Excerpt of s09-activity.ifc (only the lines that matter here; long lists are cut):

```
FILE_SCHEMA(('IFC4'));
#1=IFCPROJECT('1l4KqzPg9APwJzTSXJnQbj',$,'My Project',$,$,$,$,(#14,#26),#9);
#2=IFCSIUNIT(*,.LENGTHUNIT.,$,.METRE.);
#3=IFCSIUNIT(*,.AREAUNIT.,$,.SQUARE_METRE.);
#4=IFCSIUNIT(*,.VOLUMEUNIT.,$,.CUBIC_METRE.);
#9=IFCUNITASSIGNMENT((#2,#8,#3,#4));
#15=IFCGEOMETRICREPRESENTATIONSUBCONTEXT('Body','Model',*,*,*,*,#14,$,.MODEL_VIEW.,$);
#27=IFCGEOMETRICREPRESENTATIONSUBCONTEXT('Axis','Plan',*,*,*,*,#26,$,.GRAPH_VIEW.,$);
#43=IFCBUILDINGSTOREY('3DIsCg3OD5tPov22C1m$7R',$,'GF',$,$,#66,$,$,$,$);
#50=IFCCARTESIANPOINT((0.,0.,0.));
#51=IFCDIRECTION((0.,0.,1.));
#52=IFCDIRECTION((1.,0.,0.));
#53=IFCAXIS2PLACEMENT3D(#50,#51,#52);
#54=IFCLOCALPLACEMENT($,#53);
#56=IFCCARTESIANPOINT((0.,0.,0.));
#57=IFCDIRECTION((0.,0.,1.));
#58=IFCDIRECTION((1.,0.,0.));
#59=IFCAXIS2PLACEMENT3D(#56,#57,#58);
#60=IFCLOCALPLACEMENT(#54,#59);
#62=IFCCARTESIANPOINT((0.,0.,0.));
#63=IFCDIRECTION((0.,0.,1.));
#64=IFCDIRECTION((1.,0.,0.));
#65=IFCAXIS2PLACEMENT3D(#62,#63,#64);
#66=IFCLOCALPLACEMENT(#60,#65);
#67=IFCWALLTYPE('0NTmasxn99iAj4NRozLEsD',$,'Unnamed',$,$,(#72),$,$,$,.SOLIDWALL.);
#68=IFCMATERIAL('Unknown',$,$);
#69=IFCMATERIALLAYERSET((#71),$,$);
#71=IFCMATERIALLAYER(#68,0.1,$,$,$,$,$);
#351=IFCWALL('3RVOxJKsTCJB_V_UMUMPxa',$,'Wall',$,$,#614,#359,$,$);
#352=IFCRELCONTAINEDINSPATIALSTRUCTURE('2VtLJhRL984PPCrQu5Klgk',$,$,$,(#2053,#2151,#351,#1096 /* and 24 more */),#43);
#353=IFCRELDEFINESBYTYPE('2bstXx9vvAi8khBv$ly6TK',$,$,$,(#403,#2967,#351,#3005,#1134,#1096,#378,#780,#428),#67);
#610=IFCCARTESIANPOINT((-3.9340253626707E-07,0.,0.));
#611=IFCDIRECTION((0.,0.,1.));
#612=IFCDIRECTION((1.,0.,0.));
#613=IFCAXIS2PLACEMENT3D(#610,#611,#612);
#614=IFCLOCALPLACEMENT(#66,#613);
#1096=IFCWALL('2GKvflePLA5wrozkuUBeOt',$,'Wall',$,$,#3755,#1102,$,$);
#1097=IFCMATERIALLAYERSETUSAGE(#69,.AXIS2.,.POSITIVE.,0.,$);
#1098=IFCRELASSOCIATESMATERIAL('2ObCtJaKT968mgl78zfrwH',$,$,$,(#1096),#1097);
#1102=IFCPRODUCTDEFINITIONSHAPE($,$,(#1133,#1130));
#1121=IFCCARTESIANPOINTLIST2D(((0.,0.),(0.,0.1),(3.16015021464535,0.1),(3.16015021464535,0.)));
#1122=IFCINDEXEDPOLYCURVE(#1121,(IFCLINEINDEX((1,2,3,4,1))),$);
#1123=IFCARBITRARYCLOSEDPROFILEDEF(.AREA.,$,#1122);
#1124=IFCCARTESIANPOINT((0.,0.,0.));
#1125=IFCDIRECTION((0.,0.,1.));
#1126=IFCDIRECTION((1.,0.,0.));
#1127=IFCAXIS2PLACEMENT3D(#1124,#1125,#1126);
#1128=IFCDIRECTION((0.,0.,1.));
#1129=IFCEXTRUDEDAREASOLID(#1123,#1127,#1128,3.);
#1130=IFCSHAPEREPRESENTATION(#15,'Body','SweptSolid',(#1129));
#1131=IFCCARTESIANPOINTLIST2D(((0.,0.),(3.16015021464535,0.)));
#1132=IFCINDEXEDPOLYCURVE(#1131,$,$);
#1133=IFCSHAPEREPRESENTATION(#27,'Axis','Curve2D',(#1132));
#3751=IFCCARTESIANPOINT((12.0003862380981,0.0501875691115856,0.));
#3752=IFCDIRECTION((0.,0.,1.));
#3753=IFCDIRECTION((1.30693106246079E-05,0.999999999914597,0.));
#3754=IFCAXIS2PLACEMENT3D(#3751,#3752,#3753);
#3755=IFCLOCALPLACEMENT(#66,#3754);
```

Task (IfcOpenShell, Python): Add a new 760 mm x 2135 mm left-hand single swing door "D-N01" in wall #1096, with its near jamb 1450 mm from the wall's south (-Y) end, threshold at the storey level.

```python
import numpy as np
import ifcopenshell
import ifcopenshell.api.feature
import ifcopenshell.api.geometry
import ifcopenshell.api.root
import ifcopenshell.api.spatial
import ifcopenshell.geom
import ifcopenshell.util.element
import ifcopenshell.util.placement
import ifcopenshell.util.representation
import ifcopenshell.util.shape
import ifcopenshell.util.unit

model = ifcopenshell.open("s09-activity.ifc")
unit_scale = ifcopenshell.util.unit.calculate_unit_scale(model)
settings = ifcopenshell.geom.settings()


def volume(element):
    """Net volume in cubic metres, openings subtracted."""
    shape = ifcopenshell.geom.create_shape(settings, element)
    return ifcopenshell.util.shape.get_volume(shape.geometry)


wall = model.by_guid("2GKvflePLA5wrozkuUBeOt")
storey = ifcopenshell.util.element.get_container(wall, ifc_class="IfcBuildingStorey")
context = ifcopenshell.util.representation.get_context(model, "Model", "Body", "MODEL_VIEW")
before = volume(wall)

width, height, from_end, sill = 0.76, 2.135, 1.45, 0.0  # metres

# The wall runs along its own X axis, and the end named is its -X end.
wall_shape = ifcopenshell.geom.create_shape(settings, wall)
x, y, z = ifcopenshell.util.shape.get_vertices(wall_shape.geometry).T
start = x.min() + from_end
face, thickness = float(y.min()), float(y.max() - y.min())
wall_matrix = ifcopenshell.util.placement.get_local_placement(wall.ObjectPlacement)
level = ifcopenshell.util.placement.get_local_placement(storey.ObjectPlacement)[2, 3]


def in_wall(x, y):
    """Placement at x, y metres in the wall's axes, at sill height."""
    matrix = wall_matrix.copy()
    matrix[:, 3] = wall_matrix @ np.array([x / unit_scale, y / unit_scale, 0.0, 1.0])
    matrix[2, 3] = level + sill / unit_scale
    return matrix


# Opening: a box that overshoots both wall faces by 50 mm.
opening = ifcopenshell.api.root.create_entity(model, ifc_class="IfcOpeningElement", predefined_type="OPENING")
box = ifcopenshell.api.geometry.add_wall_representation(
    model, context=context, length=width, height=height, thickness=thickness + 0.1
)
ifcopenshell.api.geometry.assign_representation(model, product=opening, representation=box)
ifcopenshell.api.geometry.edit_object_placement(model, product=opening, matrix=in_wall(start, face - 0.05), is_si=False)
ifcopenshell.api.feature.add_feature(model, feature=opening, element=wall)

door = ifcopenshell.api.root.create_entity(model, ifc_class="IfcDoor", name="D-N01", predefined_type="DOOR")
door.OverallWidth, door.OverallHeight = width / unit_scale, height / unit_scale
door.OperationType = "SINGLE_SWING_LEFT"
body = ifcopenshell.api.geometry.add_door_representation(
    model,
    context=context,
    overall_width=door.OverallWidth,
    overall_height=door.OverallHeight,
    operation_type="SINGLE_SWING_LEFT",
    lining_properties={"LiningDepth": thickness / unit_scale, "ThresholdDepth": thickness / unit_scale},
)
ifcopenshell.api.geometry.assign_representation(model, product=door, representation=body)
ifcopenshell.api.spatial.assign_container(model, products=[door], relating_structure=storey)
ifcopenshell.api.feature.add_filling(model, opening=opening, element=door)

# The lining spans the wall, so the door starts at the wall face.
ifcopenshell.api.geometry.edit_object_placement(model, product=door, matrix=in_wall(start, face), is_si=False)

after = volume(wall)

print(f"wall volume {before:.3f} -> {after:.3f} m3")

model.write("s09-activity-out.ifc")
```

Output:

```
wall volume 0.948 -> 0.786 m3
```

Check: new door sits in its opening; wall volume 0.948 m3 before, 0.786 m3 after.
